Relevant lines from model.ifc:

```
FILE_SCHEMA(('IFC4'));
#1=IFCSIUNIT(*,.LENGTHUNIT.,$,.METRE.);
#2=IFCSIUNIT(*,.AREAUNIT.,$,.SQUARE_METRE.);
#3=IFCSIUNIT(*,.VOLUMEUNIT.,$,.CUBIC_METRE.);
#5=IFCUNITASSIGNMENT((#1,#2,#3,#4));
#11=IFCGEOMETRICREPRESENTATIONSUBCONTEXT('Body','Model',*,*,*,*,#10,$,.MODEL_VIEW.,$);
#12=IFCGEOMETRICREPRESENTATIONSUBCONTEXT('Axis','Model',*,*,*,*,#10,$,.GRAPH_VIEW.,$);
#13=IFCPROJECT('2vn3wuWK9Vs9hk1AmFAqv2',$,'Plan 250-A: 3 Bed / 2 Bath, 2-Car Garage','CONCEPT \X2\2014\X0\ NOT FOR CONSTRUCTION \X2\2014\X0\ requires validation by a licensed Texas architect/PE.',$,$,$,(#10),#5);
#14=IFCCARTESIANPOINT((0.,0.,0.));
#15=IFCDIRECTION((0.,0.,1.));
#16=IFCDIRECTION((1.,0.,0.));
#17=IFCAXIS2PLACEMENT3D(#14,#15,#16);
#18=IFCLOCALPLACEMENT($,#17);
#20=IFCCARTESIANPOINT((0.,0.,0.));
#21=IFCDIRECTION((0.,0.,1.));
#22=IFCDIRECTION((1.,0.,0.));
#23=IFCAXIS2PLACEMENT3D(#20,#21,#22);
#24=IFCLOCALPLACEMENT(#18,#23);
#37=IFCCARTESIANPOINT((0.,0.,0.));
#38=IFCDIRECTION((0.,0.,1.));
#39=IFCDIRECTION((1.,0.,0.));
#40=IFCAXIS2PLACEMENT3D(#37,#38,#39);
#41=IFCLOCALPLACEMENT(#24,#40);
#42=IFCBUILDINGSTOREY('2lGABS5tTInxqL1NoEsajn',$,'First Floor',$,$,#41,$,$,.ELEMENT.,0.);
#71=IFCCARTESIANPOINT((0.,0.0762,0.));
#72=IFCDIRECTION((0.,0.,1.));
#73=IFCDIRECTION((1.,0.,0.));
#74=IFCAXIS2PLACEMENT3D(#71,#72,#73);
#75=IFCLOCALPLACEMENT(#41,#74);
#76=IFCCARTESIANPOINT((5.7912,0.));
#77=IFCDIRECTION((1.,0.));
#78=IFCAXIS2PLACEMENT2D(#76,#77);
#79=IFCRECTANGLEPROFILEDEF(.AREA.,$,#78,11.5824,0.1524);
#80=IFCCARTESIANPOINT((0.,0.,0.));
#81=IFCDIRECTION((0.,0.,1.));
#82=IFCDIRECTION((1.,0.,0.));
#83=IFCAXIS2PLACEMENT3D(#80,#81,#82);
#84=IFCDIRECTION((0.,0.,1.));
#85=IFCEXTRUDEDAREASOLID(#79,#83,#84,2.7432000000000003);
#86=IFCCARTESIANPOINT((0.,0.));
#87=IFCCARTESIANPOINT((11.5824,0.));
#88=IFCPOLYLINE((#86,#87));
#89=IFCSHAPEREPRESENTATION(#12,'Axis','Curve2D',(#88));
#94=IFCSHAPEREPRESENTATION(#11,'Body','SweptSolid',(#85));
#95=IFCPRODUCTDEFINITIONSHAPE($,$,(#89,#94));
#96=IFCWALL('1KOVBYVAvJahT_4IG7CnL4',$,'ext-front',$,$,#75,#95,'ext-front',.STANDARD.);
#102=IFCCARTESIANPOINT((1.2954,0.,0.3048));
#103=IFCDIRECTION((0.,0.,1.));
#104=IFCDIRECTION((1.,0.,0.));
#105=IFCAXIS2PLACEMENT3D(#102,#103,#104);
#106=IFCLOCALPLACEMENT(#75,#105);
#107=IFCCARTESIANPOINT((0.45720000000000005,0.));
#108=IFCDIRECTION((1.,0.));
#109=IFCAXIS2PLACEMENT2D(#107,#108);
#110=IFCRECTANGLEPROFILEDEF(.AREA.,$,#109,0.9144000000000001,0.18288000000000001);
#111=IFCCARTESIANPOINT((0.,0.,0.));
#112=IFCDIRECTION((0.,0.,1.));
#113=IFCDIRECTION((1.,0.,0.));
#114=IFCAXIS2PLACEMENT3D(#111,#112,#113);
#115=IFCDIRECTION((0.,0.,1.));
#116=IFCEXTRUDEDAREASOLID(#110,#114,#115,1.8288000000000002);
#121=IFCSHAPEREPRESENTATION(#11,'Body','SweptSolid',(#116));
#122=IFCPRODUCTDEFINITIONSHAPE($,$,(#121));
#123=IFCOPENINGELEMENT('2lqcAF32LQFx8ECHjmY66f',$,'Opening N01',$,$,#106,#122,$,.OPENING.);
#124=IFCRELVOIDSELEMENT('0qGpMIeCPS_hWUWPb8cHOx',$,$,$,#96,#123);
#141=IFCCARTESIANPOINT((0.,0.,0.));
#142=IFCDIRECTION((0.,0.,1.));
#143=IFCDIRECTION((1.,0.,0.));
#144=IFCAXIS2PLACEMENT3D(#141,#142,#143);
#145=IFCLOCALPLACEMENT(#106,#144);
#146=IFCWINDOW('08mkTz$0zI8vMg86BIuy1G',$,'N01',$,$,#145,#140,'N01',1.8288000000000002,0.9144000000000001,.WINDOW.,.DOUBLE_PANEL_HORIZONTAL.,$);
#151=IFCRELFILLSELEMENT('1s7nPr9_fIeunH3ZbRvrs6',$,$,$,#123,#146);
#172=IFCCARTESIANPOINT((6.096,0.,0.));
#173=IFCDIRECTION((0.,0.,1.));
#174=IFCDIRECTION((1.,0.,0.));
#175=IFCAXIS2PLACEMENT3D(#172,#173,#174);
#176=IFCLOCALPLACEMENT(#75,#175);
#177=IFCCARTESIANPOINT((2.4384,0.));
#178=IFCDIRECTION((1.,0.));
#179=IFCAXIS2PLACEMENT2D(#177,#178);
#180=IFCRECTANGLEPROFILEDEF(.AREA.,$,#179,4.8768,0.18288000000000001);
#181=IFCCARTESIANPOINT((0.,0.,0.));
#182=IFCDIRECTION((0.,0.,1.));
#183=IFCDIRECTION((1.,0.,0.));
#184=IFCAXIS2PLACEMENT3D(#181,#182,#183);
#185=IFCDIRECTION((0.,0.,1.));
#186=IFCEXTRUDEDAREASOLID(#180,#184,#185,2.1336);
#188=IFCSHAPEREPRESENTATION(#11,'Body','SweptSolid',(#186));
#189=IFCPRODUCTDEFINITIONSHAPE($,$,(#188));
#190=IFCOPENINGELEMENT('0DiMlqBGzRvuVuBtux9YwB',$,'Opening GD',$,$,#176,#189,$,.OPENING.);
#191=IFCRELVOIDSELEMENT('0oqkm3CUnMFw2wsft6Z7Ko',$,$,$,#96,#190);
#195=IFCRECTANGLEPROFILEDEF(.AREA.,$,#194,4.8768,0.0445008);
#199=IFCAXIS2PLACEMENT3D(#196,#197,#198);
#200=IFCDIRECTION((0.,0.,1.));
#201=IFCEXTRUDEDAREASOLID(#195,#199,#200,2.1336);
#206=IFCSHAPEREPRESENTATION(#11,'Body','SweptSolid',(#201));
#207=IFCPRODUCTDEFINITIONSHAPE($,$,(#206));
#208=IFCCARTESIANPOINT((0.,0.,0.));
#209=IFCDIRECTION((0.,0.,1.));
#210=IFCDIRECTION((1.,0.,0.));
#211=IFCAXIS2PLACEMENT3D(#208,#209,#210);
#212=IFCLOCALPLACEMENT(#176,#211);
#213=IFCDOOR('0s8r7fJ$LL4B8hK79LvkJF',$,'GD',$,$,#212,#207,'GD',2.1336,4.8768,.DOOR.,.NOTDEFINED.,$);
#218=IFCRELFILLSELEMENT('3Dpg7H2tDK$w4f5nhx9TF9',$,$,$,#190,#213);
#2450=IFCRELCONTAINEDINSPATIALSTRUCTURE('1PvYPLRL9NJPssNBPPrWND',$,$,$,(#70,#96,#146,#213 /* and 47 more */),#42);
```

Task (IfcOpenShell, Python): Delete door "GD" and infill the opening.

```python
import ifcopenshell
import ifcopenshell.api.feature
import ifcopenshell.api.root
import ifcopenshell.geom
import ifcopenshell.util.shape

model = ifcopenshell.open("model.ifc")
settings = ifcopenshell.geom.settings()


def volume(element):
    """Net volume in cubic metres, openings subtracted."""
    shape = ifcopenshell.geom.create_shape(settings, element)
    return ifcopenshell.util.shape.get_volume(shape.geometry)


door = model.by_guid("0s8r7fJ$LL4B8hK79LvkJF")
opening = door.FillsVoids[0].RelatingOpeningElement
wall = opening.VoidsElements[0].RelatingBuildingElement
before = volume(wall)

ifcopenshell.api.root.remove_product(model, product=door)
ifcopenshell.api.feature.remove_feature(model, feature=opening)

after = volume(wall)

print(f"wall volume {before:.3f} -> {after:.3f} m3")

model.write("model_rev.ifc")
```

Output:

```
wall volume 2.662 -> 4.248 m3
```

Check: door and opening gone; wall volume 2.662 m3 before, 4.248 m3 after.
